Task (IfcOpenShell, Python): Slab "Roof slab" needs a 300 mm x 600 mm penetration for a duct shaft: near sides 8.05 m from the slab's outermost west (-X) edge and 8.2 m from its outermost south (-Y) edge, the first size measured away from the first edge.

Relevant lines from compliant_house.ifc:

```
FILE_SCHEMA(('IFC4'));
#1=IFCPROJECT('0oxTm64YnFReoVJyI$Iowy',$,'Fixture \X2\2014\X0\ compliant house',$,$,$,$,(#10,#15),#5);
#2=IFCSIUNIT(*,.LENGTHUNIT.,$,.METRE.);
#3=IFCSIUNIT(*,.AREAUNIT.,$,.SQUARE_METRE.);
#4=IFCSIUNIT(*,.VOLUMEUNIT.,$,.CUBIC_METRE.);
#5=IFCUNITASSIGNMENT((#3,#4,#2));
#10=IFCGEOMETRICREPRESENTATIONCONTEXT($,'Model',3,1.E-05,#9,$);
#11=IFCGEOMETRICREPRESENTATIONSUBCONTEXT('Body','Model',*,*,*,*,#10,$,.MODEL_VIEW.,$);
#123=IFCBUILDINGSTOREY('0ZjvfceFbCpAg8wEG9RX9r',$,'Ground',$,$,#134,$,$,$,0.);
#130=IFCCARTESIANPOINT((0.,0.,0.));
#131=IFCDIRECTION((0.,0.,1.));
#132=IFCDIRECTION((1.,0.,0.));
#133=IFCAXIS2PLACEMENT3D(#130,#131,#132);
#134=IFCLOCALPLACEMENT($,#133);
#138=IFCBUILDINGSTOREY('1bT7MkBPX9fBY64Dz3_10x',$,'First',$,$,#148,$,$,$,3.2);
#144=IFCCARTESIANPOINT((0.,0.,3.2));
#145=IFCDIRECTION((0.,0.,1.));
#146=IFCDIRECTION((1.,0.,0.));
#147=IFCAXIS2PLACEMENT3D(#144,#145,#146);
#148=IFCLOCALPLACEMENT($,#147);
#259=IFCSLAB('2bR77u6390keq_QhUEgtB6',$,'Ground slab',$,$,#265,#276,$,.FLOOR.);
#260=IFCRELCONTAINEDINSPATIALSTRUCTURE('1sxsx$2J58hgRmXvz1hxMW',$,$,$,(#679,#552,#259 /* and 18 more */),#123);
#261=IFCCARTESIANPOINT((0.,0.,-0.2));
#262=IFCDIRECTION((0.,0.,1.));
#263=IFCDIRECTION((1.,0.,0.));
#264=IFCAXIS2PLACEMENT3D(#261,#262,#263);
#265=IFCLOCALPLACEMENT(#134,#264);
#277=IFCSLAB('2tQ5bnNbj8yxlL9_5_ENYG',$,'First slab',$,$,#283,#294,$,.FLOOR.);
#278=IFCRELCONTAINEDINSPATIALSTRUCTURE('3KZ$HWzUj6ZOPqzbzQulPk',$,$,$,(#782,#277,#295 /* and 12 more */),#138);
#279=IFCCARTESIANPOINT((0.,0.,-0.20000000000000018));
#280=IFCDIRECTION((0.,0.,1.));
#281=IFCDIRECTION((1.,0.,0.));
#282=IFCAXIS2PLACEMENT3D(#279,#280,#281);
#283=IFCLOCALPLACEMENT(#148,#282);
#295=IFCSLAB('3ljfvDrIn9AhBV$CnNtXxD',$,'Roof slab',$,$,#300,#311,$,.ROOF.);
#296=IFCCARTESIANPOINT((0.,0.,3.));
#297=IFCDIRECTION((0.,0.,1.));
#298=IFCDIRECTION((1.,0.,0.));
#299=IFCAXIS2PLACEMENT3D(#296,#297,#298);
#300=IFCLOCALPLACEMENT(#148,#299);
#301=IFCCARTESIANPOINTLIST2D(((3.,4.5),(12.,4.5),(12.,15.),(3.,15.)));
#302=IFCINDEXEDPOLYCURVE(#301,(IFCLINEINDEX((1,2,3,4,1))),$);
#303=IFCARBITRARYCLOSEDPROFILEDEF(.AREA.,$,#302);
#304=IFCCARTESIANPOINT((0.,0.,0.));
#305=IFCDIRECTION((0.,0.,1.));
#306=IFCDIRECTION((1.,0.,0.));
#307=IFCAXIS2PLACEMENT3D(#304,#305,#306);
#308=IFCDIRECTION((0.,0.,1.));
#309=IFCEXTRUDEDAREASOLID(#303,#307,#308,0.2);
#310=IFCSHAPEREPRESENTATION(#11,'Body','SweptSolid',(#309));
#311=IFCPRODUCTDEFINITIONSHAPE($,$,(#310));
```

```python
import numpy as np
import ifcopenshell
import ifcopenshell.api.feature
import ifcopenshell.api.geometry
import ifcopenshell.api.root
import ifcopenshell.geom
import ifcopenshell.util.placement
import ifcopenshell.util.representation
import ifcopenshell.util.shape
import ifcopenshell.util.unit

model = ifcopenshell.open("compliant_house.ifc")
unit_scale = ifcopenshell.util.unit.calculate_unit_scale(model)
settings = ifcopenshell.geom.settings()


def volume(element):
    """Net volume in cubic metres, openings subtracted."""
    shape = ifcopenshell.geom.create_shape(settings, element)
    return ifcopenshell.util.shape.get_volume(shape.geometry)


slab = model.by_id(295)
before = volume(slab)

# Extent in the slab's own axes, in metres. The edges named are its -X and -Y sides.
slab_shape = ifcopenshell.geom.create_shape(settings, slab)
vertices = ifcopenshell.util.shape.get_vertices(slab_shape.geometry)
x_min, y_min, bottom = vertices.min(axis=0)
top = vertices[:, 2].max()

opening = ifcopenshell.api.root.create_entity(model, ifc_class="IfcOpeningElement", name="Duct shaft opening", predefined_type="OPENING")
context = ifcopenshell.util.representation.get_context(model, "Model", "Body", "MODEL_VIEW")
width, depth = 0.3, 0.6
outline = [(0.0, 0.0), (width, 0.0), (width, depth), (0.0, depth), (0.0, 0.0)]
# Overshoot both faces by 50 mm so the cut is clean.
shape = ifcopenshell.api.geometry.add_slab_representation(
    model, context=context, depth=top - bottom + 0.1, polyline=outline
)
ifcopenshell.api.geometry.assign_representation(model, product=opening, representation=shape)

matrix = ifcopenshell.util.placement.get_local_placement(slab.ObjectPlacement)
matrix[:, 3] = matrix @ np.append(np.array([x_min + 8.05, y_min + 8.2, bottom - 0.05]) / unit_scale, 1.0)
ifcopenshell.api.geometry.edit_object_placement(model, product=opening, matrix=matrix, is_si=False)
ifcopenshell.api.feature.add_feature(model, feature=opening, element=slab)

after = volume(slab)

print(f"slab volume {before:.3f} -> {after:.3f} m3")

model.write("compliant_house_v2.ifc")
```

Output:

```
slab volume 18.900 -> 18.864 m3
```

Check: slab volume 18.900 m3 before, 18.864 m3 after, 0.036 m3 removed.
